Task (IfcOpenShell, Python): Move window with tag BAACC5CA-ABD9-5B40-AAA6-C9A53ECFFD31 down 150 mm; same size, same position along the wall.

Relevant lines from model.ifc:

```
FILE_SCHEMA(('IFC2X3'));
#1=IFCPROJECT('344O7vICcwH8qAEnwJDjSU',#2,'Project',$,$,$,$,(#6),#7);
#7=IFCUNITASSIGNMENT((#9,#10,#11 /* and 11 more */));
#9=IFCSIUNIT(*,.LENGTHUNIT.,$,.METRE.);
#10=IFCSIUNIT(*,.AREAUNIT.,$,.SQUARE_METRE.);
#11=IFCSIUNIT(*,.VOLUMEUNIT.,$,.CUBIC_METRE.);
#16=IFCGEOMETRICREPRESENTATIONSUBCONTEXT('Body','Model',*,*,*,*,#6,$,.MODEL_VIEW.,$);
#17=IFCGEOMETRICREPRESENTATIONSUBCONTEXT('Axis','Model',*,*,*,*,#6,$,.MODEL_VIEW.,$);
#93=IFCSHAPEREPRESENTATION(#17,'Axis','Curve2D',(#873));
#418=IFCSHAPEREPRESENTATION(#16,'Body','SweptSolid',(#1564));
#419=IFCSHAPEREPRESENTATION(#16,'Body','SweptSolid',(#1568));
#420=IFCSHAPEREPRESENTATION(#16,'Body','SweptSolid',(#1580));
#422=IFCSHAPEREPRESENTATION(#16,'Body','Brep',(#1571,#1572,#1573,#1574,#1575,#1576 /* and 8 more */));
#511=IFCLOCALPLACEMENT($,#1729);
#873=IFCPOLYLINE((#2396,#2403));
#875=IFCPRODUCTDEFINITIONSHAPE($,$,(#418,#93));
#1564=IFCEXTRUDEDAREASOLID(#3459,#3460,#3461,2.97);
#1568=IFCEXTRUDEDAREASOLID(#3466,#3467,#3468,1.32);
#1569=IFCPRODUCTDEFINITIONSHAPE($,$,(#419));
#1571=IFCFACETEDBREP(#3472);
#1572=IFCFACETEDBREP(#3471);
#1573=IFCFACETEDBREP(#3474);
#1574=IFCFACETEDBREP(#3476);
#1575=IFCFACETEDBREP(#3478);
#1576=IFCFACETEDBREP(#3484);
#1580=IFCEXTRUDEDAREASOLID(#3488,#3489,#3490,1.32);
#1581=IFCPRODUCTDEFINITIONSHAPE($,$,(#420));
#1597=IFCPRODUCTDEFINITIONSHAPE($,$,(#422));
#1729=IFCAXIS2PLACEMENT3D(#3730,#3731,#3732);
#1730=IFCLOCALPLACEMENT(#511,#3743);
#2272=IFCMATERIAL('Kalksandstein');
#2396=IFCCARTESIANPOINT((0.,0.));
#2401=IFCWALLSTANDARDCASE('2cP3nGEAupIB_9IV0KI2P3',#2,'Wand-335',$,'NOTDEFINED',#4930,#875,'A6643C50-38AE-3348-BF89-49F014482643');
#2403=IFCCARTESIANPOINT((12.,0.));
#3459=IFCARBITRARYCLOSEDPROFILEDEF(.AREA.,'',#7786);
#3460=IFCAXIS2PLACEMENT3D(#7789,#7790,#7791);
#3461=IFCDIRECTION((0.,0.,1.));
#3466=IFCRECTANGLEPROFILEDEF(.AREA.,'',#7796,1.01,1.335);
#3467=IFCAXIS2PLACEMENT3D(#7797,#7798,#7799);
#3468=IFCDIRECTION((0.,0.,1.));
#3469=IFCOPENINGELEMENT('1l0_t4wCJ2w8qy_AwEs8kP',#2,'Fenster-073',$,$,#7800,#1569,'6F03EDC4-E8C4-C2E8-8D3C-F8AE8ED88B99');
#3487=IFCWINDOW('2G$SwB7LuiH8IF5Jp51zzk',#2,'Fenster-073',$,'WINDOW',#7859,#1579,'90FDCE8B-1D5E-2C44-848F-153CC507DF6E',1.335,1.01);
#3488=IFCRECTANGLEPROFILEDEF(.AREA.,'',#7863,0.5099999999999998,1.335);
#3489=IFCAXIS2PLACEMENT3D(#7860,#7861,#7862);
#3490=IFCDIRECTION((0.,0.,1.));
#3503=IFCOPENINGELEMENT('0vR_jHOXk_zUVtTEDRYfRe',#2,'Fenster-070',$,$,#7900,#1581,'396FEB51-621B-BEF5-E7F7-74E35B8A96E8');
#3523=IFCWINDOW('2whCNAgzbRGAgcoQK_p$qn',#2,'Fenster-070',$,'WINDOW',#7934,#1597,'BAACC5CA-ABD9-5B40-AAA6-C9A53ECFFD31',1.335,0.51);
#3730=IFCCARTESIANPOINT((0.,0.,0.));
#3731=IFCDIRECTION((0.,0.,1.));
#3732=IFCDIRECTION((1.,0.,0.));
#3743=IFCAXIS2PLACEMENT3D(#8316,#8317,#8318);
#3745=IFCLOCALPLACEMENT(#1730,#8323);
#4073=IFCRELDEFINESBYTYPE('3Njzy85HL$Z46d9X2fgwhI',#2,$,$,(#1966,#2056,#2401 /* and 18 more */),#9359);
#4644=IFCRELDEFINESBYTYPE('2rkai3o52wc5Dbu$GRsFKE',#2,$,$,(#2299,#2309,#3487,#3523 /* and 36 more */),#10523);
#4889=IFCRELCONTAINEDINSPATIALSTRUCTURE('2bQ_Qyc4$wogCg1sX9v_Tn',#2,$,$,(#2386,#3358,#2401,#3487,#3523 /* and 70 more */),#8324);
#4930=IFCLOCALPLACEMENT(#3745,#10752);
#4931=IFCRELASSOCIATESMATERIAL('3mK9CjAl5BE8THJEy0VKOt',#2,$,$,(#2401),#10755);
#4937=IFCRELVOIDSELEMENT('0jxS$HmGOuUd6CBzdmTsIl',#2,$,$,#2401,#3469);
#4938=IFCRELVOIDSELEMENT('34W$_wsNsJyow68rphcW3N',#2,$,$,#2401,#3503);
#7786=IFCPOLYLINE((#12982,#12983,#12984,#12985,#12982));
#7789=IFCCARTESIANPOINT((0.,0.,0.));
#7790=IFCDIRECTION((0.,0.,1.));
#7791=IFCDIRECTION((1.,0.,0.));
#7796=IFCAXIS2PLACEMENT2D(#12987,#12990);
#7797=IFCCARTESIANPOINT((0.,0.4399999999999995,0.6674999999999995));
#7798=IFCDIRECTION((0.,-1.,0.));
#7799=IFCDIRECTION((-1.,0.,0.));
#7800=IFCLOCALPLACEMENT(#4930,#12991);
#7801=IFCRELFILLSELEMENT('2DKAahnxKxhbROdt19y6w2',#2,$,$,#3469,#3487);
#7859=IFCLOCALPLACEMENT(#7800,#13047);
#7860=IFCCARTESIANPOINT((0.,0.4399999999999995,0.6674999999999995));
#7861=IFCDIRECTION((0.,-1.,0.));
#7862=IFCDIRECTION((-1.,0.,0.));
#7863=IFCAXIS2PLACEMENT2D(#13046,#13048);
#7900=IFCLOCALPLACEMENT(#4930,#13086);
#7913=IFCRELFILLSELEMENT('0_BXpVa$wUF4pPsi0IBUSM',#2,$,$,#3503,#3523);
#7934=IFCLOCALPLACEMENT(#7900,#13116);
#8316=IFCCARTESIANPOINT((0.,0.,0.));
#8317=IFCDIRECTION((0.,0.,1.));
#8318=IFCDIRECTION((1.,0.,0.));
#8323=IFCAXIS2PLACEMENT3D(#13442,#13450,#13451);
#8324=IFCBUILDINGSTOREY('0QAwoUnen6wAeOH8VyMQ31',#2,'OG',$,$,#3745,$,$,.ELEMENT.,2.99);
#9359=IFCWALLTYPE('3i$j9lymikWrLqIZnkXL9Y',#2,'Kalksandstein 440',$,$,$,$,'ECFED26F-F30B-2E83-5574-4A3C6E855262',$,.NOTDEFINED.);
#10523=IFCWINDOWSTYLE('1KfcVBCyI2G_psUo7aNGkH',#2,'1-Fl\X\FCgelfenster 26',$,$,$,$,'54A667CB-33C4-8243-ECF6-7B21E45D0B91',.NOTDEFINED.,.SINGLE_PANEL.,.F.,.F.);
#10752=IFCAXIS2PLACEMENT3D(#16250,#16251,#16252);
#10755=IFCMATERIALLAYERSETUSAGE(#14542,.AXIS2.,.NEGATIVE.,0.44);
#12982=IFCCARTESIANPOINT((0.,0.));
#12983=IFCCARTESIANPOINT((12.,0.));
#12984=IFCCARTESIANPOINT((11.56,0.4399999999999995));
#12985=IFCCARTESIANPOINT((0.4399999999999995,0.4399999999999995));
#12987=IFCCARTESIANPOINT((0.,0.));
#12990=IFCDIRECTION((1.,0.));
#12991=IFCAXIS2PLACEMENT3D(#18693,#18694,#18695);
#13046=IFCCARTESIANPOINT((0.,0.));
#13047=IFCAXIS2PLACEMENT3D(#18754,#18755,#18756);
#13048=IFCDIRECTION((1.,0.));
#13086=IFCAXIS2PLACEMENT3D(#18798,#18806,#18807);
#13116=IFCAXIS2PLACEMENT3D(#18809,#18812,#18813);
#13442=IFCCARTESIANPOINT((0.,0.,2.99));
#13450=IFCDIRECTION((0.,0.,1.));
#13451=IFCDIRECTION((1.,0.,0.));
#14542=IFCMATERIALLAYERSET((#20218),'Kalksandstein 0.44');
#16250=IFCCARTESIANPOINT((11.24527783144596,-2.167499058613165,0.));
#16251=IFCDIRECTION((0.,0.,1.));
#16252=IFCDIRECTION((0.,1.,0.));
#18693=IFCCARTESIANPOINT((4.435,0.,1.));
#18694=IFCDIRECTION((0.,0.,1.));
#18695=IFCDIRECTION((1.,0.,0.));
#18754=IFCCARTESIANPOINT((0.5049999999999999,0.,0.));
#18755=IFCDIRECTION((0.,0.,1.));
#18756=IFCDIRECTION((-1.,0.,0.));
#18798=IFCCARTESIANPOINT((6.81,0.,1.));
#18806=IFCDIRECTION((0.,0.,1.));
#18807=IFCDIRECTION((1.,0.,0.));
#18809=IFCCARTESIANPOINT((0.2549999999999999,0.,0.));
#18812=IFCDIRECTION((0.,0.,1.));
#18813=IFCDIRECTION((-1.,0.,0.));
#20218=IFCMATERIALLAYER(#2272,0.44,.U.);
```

```python
import numpy as np
import ifcopenshell
import ifcopenshell.api.geometry
import ifcopenshell.util.placement
import ifcopenshell.util.unit

model = ifcopenshell.open("model.ifc")
unit_scale = ifcopenshell.util.unit.calculate_unit_scale(model)

window = model.by_guid("2whCNAgzbRGAgcoQK_p$qn")
opening = window.FillsVoids[0].RelatingOpeningElement
dz = -0.15

shift = np.array([0.0, 0.0, dz])
# The window is placed relative to its opening, so it follows when the opening moves.
matrix = ifcopenshell.util.placement.get_local_placement(opening.ObjectPlacement)
matrix[:3, 3] += shift
ifcopenshell.api.geometry.edit_object_placement(
    model, product=opening, matrix=matrix, is_si=False, should_transform_children=True
)

print(f"moved by {dz * unit_scale:+.3f} m")

model.write("model_updated.ifc")
```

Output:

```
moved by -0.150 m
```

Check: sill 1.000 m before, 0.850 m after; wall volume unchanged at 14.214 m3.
